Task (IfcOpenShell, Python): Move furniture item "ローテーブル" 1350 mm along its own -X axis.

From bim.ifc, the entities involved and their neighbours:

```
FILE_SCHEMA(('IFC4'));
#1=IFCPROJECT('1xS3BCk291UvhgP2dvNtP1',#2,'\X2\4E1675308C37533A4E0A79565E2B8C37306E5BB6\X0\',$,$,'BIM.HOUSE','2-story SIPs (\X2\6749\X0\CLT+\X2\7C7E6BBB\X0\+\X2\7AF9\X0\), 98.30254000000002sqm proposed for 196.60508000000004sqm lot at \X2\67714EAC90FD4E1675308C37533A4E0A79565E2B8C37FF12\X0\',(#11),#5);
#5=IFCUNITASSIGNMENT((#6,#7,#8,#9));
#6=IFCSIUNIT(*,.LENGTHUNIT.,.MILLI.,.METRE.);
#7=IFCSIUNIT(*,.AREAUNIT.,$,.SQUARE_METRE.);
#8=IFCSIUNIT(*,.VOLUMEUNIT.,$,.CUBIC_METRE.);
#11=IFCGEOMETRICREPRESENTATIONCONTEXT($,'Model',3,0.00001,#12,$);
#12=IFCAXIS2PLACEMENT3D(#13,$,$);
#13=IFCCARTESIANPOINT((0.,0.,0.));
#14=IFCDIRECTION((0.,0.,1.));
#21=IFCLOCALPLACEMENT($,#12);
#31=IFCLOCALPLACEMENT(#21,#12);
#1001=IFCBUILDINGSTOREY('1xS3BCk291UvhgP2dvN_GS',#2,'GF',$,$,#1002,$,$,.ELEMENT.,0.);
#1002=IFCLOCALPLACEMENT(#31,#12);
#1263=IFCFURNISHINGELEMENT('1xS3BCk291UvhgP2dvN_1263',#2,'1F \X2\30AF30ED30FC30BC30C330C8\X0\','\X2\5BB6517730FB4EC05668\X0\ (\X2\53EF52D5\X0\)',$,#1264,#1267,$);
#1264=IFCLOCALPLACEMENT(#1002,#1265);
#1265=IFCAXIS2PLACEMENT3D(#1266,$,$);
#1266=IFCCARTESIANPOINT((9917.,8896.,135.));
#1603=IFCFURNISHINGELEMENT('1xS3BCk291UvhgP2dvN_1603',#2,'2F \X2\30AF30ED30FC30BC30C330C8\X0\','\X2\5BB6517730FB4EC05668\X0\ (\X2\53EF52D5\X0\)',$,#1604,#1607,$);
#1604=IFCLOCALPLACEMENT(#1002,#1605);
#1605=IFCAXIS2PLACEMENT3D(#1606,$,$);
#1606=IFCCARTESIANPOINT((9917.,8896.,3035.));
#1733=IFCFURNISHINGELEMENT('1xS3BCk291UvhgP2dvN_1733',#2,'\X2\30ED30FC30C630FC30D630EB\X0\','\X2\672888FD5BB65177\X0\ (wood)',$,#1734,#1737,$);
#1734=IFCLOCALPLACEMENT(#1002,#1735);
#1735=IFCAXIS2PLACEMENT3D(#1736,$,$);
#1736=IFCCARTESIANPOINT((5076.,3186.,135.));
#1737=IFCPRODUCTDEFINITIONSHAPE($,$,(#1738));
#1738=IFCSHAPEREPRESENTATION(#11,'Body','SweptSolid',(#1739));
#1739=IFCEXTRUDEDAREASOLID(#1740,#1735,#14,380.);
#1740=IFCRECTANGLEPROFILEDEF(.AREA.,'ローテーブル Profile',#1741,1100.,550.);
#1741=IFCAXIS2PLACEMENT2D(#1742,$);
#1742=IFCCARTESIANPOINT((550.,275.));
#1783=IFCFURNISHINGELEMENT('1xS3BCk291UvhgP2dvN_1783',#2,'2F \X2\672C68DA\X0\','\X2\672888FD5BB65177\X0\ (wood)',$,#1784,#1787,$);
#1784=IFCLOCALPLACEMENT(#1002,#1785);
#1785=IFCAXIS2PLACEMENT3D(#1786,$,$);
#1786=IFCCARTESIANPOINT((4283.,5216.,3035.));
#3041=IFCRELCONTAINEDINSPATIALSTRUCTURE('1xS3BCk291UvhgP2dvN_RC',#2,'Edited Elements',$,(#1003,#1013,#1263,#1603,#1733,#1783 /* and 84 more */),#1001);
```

```python
import ifcopenshell
import ifcopenshell.api.geometry
import ifcopenshell.util.placement
import ifcopenshell.util.unit

model = ifcopenshell.open("bim.ifc")
unit_scale = ifcopenshell.util.unit.calculate_unit_scale(model)

item = model.by_id(1733)
matrix = ifcopenshell.util.placement.get_local_placement(item.ObjectPlacement)
matrix[:3, 3] -= matrix[:3, 0] * 1.35 / unit_scale
ifcopenshell.api.geometry.edit_object_placement(model, product=item, matrix=matrix, is_si=False)

print(ifcopenshell.util.placement.get_local_placement(item.ObjectPlacement).round(3) + 0.0)

model.write("bim_updated.ifc")
```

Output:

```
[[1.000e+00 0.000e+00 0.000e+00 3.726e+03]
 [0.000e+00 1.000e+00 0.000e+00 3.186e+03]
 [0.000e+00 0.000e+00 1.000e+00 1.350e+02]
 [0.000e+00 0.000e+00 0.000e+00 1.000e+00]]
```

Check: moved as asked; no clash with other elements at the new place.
